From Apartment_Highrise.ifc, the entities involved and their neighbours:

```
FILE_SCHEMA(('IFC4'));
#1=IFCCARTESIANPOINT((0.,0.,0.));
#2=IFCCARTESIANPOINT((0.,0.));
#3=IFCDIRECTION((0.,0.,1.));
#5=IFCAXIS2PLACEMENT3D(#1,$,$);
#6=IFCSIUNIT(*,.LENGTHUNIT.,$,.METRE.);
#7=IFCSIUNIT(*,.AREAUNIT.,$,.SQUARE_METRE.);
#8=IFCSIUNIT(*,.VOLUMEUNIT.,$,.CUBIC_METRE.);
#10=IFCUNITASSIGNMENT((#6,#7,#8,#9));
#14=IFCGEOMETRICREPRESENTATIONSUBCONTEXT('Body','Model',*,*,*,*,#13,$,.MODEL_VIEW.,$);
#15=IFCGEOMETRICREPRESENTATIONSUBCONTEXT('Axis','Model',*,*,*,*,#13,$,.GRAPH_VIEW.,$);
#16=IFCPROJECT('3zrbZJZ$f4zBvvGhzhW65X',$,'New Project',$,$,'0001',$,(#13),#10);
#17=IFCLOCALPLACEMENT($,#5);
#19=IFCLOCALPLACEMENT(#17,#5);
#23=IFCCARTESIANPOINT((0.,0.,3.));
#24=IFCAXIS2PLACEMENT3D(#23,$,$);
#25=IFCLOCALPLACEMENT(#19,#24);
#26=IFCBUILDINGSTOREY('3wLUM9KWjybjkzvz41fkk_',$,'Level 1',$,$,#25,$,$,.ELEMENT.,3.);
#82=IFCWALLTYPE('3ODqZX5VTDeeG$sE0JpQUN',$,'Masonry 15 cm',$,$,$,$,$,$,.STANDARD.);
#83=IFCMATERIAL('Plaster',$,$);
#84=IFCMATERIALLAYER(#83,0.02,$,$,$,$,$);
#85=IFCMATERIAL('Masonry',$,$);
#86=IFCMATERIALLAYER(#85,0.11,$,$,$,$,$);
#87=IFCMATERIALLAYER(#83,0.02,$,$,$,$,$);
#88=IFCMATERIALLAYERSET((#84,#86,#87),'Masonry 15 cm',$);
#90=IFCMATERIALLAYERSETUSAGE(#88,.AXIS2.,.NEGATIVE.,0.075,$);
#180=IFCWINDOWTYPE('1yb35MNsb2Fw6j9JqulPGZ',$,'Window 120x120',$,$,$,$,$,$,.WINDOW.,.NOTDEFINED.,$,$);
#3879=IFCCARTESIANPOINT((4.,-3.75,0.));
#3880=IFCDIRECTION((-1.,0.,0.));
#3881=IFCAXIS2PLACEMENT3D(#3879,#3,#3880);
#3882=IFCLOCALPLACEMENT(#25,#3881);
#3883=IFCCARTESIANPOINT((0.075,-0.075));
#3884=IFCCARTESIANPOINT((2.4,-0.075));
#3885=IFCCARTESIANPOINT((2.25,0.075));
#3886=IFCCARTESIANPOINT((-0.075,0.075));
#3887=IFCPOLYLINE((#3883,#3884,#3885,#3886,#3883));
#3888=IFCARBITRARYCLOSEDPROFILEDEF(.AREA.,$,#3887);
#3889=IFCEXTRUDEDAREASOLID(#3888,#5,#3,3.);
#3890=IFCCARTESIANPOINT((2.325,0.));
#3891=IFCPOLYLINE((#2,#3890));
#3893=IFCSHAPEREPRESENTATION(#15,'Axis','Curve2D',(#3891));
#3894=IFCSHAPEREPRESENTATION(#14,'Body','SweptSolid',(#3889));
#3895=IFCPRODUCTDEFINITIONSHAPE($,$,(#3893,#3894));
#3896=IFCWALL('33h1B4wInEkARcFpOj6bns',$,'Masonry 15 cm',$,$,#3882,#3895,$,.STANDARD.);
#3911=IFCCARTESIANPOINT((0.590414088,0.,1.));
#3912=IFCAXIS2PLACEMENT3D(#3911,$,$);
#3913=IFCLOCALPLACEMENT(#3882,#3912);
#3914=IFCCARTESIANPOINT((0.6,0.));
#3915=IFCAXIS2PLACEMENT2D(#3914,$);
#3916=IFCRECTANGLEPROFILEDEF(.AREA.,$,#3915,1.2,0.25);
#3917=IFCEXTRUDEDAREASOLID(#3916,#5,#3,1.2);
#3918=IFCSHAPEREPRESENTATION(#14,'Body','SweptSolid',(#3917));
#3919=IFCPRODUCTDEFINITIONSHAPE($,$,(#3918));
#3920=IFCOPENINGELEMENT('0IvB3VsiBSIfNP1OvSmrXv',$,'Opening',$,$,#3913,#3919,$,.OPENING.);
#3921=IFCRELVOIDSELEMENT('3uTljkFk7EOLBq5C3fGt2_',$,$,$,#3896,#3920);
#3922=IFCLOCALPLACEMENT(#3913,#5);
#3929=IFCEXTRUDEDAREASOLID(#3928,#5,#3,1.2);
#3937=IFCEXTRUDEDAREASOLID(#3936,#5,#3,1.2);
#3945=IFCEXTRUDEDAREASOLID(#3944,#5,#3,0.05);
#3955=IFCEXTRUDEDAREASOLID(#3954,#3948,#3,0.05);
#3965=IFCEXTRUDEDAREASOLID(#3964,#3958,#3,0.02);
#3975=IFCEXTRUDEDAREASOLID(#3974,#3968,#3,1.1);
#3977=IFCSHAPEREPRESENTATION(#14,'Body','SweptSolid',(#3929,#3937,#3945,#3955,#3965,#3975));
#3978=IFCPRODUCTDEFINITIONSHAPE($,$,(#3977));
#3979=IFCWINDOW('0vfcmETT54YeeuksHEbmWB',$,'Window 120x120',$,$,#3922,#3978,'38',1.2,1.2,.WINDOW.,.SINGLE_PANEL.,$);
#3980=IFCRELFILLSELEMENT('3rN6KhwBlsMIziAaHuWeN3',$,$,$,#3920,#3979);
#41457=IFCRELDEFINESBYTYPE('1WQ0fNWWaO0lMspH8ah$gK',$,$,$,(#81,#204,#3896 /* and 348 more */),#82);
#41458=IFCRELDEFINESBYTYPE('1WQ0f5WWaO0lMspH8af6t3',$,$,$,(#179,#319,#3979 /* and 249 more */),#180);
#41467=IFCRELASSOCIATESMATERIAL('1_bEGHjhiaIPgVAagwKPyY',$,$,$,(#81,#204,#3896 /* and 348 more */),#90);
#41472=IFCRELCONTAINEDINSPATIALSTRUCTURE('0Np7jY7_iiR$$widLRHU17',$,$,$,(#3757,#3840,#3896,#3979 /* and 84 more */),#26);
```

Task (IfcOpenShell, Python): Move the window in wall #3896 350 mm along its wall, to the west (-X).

```python
import ifcopenshell
import ifcopenshell.api.geometry
import ifcopenshell.util.placement
import ifcopenshell.util.unit

model = ifcopenshell.open("Apartment_Highrise.ifc")
unit_scale = ifcopenshell.util.unit.calculate_unit_scale(model)

window = model.by_id(3979)
opening = window.FillsVoids[0].RelatingOpeningElement
wall = opening.VoidsElements[0].RelatingBuildingElement

wall_matrix = ifcopenshell.util.placement.get_local_placement(wall.ObjectPlacement)
shift = wall_matrix[:3, 0] * 0.35 / unit_scale
before = ifcopenshell.util.placement.get_local_placement(window.ObjectPlacement)[:3, 3].copy()

# The window is placed relative to its opening, so it follows when the opening moves.
matrix = ifcopenshell.util.placement.get_local_placement(opening.ObjectPlacement)
matrix[:3, 3] += shift
ifcopenshell.api.geometry.edit_object_placement(
    model, product=opening, matrix=matrix, is_si=False, should_transform_children=True
)

after = ifcopenshell.util.placement.get_local_placement(window.ObjectPlacement)[:3, 3]
print("window moved by", (after - before).round(3) + 0.0)

model.write("Apartment_Highrise_rev.ifc")
```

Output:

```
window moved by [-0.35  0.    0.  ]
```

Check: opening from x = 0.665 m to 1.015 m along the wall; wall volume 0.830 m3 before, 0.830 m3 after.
